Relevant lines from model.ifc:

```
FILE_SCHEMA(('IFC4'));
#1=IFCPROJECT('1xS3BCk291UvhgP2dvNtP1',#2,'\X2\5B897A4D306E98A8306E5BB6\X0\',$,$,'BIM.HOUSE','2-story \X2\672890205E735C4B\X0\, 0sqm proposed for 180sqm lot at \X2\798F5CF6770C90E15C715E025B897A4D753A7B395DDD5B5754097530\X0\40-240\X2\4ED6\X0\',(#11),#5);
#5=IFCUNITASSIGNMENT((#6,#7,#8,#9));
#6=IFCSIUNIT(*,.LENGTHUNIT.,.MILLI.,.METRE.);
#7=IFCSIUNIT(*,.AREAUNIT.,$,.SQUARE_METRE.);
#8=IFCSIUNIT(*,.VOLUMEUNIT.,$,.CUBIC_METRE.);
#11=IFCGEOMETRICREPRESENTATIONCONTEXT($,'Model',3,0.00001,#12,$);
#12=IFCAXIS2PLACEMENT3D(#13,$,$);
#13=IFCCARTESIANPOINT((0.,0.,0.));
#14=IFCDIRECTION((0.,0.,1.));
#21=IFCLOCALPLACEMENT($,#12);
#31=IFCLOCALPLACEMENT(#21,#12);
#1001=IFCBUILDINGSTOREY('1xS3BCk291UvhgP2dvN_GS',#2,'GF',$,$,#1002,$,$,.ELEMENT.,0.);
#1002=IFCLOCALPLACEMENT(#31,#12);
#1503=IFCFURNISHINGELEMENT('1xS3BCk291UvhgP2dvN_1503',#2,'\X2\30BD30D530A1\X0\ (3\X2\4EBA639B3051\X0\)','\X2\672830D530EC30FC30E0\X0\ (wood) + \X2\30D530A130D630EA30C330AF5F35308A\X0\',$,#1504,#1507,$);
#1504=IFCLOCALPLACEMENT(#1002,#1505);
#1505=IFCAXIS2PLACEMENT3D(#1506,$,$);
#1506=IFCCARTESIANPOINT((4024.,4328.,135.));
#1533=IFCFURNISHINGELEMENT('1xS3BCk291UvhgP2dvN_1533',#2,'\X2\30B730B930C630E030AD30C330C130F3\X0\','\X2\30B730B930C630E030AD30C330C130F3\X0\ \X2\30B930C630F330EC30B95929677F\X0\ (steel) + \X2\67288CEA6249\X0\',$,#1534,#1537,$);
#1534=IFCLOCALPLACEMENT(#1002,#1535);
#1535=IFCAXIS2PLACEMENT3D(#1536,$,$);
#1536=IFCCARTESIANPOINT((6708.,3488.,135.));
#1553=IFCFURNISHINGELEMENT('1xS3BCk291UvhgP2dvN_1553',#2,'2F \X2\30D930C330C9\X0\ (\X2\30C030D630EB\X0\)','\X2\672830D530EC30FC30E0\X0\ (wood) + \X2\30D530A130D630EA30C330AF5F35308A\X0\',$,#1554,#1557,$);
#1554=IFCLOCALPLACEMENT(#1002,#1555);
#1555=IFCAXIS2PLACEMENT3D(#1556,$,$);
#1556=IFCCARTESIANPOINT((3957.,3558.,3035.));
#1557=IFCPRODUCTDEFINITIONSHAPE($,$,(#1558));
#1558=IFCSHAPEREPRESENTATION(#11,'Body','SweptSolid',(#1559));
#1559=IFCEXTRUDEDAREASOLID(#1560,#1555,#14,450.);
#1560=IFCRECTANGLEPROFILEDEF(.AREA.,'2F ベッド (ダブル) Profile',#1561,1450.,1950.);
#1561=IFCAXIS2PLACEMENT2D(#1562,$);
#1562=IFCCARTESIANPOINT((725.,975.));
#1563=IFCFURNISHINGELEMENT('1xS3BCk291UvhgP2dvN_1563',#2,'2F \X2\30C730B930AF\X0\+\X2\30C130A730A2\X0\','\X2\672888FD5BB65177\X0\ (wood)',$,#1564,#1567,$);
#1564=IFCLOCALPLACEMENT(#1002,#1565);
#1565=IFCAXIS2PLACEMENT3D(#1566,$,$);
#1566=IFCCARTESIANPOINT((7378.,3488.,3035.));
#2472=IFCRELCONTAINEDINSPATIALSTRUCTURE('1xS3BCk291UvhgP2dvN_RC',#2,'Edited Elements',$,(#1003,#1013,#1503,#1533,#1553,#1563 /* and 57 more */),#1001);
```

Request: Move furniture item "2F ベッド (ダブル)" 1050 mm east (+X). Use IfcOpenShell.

```python
import ifcopenshell
import ifcopenshell.api.geometry
import ifcopenshell.util.placement
import ifcopenshell.util.unit

model = ifcopenshell.open("model.ifc")
unit_scale = ifcopenshell.util.unit.calculate_unit_scale(model)

item = model.by_id(1553)
matrix = ifcopenshell.util.placement.get_local_placement(item.ObjectPlacement)
matrix[0, 3] += 1.05 / unit_scale
ifcopenshell.api.geometry.edit_object_placement(model, product=item, matrix=matrix, is_si=False)

print(ifcopenshell.util.placement.get_local_placement(item.ObjectPlacement).round(3) + 0.0)

model.write("model_edited.ifc")
```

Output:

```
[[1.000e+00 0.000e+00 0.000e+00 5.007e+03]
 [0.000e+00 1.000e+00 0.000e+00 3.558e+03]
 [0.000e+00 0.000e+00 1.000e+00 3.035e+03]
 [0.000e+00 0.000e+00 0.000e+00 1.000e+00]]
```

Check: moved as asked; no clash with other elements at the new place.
